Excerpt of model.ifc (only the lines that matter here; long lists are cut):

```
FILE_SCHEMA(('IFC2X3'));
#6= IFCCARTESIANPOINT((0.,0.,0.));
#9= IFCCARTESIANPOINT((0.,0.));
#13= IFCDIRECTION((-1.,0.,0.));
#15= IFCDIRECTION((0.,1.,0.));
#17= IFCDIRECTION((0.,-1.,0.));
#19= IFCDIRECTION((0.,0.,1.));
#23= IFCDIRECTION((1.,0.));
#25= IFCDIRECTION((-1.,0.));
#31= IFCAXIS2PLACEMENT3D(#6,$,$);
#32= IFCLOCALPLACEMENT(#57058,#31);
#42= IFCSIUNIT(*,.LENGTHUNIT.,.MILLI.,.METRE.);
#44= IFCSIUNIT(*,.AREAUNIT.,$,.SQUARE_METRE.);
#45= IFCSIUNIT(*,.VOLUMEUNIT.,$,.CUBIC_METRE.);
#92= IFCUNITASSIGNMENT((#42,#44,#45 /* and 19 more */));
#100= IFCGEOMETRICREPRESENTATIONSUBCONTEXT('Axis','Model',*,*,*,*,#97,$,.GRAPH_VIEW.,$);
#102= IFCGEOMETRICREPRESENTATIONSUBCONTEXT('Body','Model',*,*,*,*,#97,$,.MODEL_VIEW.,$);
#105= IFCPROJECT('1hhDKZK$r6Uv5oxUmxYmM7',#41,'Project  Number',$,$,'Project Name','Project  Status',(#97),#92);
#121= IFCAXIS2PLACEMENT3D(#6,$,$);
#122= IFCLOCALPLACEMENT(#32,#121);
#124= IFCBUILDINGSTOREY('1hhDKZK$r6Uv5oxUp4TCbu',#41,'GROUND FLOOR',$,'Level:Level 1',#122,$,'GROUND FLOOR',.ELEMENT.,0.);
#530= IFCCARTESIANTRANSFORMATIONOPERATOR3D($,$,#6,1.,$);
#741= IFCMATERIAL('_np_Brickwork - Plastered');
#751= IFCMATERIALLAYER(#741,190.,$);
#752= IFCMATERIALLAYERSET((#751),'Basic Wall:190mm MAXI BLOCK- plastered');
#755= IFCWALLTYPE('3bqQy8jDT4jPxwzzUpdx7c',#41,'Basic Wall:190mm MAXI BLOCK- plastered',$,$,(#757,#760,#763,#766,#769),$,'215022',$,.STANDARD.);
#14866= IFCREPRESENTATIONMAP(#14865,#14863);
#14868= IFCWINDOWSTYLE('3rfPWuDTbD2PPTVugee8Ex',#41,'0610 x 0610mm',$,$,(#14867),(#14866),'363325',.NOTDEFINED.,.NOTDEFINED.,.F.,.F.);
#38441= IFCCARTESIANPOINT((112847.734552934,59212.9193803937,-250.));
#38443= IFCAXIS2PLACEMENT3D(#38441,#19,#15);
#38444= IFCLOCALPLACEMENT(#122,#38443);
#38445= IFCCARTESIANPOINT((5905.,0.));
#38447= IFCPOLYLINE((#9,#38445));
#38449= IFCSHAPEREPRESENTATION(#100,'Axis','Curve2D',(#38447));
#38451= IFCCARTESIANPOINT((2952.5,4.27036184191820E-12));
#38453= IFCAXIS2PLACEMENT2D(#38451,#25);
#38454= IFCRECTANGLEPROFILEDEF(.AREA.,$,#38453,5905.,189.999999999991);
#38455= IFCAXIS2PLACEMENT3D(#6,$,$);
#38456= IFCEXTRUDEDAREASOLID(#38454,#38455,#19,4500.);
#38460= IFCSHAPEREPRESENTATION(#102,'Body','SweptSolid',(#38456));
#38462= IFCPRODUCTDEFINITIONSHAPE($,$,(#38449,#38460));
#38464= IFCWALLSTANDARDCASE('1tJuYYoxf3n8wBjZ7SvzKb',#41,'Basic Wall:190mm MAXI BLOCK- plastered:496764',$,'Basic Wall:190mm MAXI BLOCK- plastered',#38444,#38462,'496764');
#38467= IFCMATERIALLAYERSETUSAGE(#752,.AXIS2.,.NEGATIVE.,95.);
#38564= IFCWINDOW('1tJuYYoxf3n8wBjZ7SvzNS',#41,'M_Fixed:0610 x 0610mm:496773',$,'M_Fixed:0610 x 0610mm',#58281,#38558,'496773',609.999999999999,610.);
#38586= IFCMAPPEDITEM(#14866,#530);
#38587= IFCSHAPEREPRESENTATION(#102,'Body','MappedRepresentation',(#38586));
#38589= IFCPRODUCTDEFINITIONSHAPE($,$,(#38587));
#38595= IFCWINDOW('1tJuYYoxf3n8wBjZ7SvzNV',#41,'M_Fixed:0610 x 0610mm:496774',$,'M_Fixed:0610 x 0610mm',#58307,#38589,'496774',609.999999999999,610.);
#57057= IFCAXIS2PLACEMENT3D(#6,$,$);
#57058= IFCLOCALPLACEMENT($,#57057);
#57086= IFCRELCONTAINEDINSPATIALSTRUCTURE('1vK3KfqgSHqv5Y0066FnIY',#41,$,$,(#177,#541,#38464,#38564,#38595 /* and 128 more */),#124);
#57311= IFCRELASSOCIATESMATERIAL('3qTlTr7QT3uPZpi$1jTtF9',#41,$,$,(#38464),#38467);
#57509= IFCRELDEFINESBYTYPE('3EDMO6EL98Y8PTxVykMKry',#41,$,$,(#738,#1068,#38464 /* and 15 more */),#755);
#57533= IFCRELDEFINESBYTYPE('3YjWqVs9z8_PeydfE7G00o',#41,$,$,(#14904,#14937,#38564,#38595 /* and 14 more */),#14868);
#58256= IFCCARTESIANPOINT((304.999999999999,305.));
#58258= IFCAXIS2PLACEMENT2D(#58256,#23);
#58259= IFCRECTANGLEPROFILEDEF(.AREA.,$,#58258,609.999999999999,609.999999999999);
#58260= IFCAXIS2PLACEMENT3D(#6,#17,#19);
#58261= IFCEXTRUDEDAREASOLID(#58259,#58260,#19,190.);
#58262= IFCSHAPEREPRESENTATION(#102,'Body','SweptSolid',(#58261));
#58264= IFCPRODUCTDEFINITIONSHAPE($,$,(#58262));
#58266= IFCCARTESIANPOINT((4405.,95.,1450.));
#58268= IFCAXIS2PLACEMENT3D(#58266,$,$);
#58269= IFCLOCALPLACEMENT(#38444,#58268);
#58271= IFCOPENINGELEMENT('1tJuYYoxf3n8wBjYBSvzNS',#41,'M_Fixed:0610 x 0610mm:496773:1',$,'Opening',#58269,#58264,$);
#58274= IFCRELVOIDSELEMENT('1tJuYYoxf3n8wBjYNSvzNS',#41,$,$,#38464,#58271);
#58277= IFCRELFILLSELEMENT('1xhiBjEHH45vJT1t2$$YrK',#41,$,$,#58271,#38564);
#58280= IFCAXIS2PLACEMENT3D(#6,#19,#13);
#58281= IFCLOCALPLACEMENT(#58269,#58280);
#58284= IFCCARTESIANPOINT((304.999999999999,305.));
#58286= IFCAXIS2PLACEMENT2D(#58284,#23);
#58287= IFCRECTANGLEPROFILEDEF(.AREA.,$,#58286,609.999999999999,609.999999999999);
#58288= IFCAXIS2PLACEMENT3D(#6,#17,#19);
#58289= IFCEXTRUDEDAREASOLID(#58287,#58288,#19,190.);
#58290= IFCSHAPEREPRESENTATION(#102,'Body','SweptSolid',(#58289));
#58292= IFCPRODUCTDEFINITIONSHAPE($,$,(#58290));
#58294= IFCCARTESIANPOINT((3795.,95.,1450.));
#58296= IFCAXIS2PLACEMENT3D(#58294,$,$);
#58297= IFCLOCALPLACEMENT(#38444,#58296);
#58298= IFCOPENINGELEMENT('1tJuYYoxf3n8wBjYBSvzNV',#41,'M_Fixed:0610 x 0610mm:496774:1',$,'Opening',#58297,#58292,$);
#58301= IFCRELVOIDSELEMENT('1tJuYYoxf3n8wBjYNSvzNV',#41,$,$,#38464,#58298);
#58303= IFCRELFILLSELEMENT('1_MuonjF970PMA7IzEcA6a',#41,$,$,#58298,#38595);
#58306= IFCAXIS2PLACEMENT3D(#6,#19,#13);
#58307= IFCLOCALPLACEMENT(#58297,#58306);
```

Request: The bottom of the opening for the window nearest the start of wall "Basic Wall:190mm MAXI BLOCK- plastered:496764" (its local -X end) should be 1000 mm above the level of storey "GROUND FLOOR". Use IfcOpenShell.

```python
import numpy as np
import ifcopenshell
import ifcopenshell.api.geometry
import ifcopenshell.geom
import ifcopenshell.util.element
import ifcopenshell.util.placement
import ifcopenshell.util.shape
import ifcopenshell.util.unit

model = ifcopenshell.open("model.ifc")
unit_scale = ifcopenshell.util.unit.calculate_unit_scale(model)

window = model.by_id(38595)
opening = window.FillsVoids[0].RelatingOpeningElement
storey = ifcopenshell.util.element.get_container(window, ifc_class="IfcBuildingStorey")
level = ifcopenshell.util.placement.get_local_placement(storey.ObjectPlacement)[2, 3]

# The opening's origin need not be at the sill, so measure its lowest point.
shape = ifcopenshell.geom.create_shape(ifcopenshell.geom.settings(), opening)
bottom = ifcopenshell.util.shape.get_shape_bottom_elevation(shape, shape.geometry) / unit_scale
dz = level + 1 / unit_scale - bottom

shift = np.array([0.0, 0.0, dz])
# The window is placed relative to its opening, so it follows when the opening moves.
matrix = ifcopenshell.util.placement.get_local_placement(opening.ObjectPlacement)
matrix[:3, 3] += shift
ifcopenshell.api.geometry.edit_object_placement(
    model, product=opening, matrix=matrix, is_si=False, should_transform_children=True
)

print(f"moved by {dz * unit_scale:+.3f} m")

model.write("model_rev.ifc")
```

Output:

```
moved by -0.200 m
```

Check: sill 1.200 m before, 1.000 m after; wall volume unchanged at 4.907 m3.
